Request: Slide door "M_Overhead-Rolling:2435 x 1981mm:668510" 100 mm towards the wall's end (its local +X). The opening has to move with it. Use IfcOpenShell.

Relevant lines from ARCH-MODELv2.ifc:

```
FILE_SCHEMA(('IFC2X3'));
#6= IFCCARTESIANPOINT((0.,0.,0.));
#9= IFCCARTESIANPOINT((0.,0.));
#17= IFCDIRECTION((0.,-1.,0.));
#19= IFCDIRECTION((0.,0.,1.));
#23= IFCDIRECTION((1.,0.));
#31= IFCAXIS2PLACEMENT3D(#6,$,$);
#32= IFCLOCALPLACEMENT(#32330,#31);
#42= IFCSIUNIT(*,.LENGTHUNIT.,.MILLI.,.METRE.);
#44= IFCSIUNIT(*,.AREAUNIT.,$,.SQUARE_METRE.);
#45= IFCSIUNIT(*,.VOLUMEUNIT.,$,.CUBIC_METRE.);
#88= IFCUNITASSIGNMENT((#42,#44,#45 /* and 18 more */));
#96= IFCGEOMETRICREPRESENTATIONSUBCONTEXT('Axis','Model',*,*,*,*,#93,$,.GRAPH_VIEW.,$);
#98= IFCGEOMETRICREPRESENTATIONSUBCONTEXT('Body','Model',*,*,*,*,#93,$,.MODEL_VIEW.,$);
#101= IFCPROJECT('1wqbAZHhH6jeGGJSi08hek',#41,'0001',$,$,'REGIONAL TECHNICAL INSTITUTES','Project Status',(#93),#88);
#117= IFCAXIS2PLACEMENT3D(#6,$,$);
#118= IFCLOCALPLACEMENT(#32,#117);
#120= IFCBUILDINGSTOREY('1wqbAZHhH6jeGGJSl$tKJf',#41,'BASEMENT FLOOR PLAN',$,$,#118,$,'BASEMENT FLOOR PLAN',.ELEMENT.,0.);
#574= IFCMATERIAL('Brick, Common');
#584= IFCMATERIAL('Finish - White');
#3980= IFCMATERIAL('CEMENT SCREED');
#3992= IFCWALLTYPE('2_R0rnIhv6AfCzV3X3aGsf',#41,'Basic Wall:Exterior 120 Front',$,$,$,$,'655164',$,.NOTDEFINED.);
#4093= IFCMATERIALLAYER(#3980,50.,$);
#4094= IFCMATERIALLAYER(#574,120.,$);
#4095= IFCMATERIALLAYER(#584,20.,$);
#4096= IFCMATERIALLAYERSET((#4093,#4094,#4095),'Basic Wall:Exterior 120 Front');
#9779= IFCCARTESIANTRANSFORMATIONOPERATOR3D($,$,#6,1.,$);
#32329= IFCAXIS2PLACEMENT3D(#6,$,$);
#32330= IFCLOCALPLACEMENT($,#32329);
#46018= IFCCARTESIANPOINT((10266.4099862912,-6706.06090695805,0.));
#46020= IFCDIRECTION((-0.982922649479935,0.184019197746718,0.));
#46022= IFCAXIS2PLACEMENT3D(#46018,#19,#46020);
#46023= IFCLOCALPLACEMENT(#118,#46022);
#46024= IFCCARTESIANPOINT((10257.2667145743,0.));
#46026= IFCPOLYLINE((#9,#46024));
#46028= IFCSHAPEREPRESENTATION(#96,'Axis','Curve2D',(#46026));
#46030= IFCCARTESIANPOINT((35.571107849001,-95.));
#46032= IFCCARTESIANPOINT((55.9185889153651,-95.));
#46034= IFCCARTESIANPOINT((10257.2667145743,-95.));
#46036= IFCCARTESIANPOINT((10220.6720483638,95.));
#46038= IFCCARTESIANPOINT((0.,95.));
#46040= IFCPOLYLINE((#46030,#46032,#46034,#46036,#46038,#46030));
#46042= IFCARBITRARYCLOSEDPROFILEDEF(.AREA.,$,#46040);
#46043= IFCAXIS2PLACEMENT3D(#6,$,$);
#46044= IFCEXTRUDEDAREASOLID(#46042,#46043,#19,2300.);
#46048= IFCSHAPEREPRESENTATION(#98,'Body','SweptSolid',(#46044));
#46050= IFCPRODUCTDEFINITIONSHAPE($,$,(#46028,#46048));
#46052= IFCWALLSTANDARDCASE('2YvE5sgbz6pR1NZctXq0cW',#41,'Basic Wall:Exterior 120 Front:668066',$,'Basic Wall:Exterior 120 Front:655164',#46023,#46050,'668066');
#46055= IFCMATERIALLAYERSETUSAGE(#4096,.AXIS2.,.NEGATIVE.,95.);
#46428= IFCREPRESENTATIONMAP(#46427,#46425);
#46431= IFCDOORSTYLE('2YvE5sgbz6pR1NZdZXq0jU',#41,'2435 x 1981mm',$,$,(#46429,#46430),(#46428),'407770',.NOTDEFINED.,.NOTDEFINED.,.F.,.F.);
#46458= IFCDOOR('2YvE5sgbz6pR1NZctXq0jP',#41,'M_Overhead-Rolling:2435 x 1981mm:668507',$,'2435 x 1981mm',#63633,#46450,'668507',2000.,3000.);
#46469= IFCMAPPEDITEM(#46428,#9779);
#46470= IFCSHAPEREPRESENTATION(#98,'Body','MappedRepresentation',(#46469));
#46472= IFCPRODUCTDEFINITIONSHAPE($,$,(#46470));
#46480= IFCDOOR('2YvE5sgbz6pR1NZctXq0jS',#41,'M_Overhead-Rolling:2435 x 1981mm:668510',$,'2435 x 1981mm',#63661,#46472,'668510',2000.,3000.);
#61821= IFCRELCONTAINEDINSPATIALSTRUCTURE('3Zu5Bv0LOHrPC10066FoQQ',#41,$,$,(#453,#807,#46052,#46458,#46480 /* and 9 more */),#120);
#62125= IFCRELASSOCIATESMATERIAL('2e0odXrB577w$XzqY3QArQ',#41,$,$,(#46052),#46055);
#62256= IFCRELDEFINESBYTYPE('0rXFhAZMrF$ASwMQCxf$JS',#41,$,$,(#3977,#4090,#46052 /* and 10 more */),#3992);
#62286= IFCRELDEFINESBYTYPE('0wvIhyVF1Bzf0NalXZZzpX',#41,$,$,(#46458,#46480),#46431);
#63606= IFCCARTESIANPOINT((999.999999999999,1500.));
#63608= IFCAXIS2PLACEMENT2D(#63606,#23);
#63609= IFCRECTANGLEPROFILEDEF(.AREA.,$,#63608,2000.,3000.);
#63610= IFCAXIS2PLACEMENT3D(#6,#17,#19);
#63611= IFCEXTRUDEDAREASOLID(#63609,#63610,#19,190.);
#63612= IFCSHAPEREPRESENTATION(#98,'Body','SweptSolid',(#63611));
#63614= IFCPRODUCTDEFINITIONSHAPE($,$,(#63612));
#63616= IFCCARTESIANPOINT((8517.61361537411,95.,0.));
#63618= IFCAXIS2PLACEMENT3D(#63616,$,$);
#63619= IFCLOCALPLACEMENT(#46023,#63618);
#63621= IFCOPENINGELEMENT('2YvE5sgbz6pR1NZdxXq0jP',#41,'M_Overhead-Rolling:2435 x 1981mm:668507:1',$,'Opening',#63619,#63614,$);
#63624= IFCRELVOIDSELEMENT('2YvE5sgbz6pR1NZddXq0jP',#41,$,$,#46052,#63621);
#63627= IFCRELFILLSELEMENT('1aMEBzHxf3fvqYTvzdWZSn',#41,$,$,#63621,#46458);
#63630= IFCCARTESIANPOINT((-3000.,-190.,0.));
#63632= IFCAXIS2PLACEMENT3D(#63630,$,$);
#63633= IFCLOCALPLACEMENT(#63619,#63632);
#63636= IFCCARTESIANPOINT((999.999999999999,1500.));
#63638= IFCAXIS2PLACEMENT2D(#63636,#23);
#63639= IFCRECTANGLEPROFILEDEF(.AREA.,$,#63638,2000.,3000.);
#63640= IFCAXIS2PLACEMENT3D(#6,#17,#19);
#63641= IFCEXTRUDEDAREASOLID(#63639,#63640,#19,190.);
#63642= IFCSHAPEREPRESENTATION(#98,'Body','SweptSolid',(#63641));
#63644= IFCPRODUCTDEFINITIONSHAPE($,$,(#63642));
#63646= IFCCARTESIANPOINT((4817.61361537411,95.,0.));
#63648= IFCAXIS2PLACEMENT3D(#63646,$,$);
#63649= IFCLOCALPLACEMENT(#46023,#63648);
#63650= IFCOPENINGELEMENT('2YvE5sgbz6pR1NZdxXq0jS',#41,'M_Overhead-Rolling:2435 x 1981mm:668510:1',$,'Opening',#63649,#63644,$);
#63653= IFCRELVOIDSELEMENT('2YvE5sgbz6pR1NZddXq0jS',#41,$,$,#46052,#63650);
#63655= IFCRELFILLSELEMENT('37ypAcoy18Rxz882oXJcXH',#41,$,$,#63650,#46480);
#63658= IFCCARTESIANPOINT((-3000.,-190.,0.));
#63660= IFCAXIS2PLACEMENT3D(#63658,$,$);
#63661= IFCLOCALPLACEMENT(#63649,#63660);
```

```python
import ifcopenshell
import ifcopenshell.api.geometry
import ifcopenshell.util.placement
import ifcopenshell.util.unit

model = ifcopenshell.open("ARCH-MODELv2.ifc")
unit_scale = ifcopenshell.util.unit.calculate_unit_scale(model)

door = model.by_guid("2YvE5sgbz6pR1NZctXq0jS")
opening = door.FillsVoids[0].RelatingOpeningElement
wall = opening.VoidsElements[0].RelatingBuildingElement

wall_matrix = ifcopenshell.util.placement.get_local_placement(wall.ObjectPlacement)
shift = wall_matrix[:3, 0] * 0.1 / unit_scale
before = ifcopenshell.util.placement.get_local_placement(door.ObjectPlacement)[:3, 3].copy()

# The door is placed relative to its opening, so it follows when the opening moves.
matrix = ifcopenshell.util.placement.get_local_placement(opening.ObjectPlacement)
matrix[:3, 3] += shift
ifcopenshell.api.geometry.edit_object_placement(
    model, product=opening, matrix=matrix, is_si=False, should_transform_children=True
)

after = ifcopenshell.util.placement.get_local_placement(door.ObjectPlacement)[:3, 3]
print("door moved by", (after - before).round(3) + 0.0)

model.write("ARCH-MODELv2_updated.ifc")
```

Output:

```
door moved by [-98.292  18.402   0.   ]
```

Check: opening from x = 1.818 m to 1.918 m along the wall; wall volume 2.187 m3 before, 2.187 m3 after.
